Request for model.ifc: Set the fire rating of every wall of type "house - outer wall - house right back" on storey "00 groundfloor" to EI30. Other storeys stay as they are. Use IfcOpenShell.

First a look at what the model holds.

```python
import ifcopenshell
import ifcopenshell.util.element

model = ifcopenshell.open("model.ifc")
print(model.schema)
storey = next(s for s in model.by_type("IfcBuildingStorey") if s.Name == "00 groundfloor")
walls = [e for e in ifcopenshell.util.element.get_decomposition(storey) if e.is_a("IfcWall")]
seen = {}
for e in walls:
    element_type = ifcopenshell.util.element.get_type(e)
    key = (element_type.Name if element_type != e and element_type else None, ifcopenshell.util.element.get_pset(e, "Pset_WallCommon", "FireRating"))
    seen[key] = seen.get(key, 0) + 1
for (name, value), count in sorted(seen.items(), key=str):
    print(count, "x", name, "|", value)
```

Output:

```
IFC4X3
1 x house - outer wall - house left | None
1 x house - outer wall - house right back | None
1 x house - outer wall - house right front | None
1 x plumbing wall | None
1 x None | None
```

```python
import ifcopenshell
import ifcopenshell.api.pset
import ifcopenshell.util.element

model = ifcopenshell.open("model.ifc")

storey = next(s for s in model.by_type("IfcBuildingStorey") if s.Name == "00 groundfloor")
walls = [e for e in ifcopenshell.util.element.get_decomposition(storey) if e.is_a("IfcWall")]

count = 0
for e in walls:
    element_type = ifcopenshell.util.element.get_type(e)
    if element_type in (None, e) or element_type.Name != "house - outer wall - house right back":
        continue
    # add_pset returns the element's existing set when there is one.
    pset = ifcopenshell.api.pset.add_pset(model, product=e, name="Pset_WallCommon")
    ifcopenshell.api.pset.edit_pset(model, pset=pset, properties={"FireRating": "EI30"})
    count += 1

print(count, "walls updated")

model.write("model-out.ifc")
```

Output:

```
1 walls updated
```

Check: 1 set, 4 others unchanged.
